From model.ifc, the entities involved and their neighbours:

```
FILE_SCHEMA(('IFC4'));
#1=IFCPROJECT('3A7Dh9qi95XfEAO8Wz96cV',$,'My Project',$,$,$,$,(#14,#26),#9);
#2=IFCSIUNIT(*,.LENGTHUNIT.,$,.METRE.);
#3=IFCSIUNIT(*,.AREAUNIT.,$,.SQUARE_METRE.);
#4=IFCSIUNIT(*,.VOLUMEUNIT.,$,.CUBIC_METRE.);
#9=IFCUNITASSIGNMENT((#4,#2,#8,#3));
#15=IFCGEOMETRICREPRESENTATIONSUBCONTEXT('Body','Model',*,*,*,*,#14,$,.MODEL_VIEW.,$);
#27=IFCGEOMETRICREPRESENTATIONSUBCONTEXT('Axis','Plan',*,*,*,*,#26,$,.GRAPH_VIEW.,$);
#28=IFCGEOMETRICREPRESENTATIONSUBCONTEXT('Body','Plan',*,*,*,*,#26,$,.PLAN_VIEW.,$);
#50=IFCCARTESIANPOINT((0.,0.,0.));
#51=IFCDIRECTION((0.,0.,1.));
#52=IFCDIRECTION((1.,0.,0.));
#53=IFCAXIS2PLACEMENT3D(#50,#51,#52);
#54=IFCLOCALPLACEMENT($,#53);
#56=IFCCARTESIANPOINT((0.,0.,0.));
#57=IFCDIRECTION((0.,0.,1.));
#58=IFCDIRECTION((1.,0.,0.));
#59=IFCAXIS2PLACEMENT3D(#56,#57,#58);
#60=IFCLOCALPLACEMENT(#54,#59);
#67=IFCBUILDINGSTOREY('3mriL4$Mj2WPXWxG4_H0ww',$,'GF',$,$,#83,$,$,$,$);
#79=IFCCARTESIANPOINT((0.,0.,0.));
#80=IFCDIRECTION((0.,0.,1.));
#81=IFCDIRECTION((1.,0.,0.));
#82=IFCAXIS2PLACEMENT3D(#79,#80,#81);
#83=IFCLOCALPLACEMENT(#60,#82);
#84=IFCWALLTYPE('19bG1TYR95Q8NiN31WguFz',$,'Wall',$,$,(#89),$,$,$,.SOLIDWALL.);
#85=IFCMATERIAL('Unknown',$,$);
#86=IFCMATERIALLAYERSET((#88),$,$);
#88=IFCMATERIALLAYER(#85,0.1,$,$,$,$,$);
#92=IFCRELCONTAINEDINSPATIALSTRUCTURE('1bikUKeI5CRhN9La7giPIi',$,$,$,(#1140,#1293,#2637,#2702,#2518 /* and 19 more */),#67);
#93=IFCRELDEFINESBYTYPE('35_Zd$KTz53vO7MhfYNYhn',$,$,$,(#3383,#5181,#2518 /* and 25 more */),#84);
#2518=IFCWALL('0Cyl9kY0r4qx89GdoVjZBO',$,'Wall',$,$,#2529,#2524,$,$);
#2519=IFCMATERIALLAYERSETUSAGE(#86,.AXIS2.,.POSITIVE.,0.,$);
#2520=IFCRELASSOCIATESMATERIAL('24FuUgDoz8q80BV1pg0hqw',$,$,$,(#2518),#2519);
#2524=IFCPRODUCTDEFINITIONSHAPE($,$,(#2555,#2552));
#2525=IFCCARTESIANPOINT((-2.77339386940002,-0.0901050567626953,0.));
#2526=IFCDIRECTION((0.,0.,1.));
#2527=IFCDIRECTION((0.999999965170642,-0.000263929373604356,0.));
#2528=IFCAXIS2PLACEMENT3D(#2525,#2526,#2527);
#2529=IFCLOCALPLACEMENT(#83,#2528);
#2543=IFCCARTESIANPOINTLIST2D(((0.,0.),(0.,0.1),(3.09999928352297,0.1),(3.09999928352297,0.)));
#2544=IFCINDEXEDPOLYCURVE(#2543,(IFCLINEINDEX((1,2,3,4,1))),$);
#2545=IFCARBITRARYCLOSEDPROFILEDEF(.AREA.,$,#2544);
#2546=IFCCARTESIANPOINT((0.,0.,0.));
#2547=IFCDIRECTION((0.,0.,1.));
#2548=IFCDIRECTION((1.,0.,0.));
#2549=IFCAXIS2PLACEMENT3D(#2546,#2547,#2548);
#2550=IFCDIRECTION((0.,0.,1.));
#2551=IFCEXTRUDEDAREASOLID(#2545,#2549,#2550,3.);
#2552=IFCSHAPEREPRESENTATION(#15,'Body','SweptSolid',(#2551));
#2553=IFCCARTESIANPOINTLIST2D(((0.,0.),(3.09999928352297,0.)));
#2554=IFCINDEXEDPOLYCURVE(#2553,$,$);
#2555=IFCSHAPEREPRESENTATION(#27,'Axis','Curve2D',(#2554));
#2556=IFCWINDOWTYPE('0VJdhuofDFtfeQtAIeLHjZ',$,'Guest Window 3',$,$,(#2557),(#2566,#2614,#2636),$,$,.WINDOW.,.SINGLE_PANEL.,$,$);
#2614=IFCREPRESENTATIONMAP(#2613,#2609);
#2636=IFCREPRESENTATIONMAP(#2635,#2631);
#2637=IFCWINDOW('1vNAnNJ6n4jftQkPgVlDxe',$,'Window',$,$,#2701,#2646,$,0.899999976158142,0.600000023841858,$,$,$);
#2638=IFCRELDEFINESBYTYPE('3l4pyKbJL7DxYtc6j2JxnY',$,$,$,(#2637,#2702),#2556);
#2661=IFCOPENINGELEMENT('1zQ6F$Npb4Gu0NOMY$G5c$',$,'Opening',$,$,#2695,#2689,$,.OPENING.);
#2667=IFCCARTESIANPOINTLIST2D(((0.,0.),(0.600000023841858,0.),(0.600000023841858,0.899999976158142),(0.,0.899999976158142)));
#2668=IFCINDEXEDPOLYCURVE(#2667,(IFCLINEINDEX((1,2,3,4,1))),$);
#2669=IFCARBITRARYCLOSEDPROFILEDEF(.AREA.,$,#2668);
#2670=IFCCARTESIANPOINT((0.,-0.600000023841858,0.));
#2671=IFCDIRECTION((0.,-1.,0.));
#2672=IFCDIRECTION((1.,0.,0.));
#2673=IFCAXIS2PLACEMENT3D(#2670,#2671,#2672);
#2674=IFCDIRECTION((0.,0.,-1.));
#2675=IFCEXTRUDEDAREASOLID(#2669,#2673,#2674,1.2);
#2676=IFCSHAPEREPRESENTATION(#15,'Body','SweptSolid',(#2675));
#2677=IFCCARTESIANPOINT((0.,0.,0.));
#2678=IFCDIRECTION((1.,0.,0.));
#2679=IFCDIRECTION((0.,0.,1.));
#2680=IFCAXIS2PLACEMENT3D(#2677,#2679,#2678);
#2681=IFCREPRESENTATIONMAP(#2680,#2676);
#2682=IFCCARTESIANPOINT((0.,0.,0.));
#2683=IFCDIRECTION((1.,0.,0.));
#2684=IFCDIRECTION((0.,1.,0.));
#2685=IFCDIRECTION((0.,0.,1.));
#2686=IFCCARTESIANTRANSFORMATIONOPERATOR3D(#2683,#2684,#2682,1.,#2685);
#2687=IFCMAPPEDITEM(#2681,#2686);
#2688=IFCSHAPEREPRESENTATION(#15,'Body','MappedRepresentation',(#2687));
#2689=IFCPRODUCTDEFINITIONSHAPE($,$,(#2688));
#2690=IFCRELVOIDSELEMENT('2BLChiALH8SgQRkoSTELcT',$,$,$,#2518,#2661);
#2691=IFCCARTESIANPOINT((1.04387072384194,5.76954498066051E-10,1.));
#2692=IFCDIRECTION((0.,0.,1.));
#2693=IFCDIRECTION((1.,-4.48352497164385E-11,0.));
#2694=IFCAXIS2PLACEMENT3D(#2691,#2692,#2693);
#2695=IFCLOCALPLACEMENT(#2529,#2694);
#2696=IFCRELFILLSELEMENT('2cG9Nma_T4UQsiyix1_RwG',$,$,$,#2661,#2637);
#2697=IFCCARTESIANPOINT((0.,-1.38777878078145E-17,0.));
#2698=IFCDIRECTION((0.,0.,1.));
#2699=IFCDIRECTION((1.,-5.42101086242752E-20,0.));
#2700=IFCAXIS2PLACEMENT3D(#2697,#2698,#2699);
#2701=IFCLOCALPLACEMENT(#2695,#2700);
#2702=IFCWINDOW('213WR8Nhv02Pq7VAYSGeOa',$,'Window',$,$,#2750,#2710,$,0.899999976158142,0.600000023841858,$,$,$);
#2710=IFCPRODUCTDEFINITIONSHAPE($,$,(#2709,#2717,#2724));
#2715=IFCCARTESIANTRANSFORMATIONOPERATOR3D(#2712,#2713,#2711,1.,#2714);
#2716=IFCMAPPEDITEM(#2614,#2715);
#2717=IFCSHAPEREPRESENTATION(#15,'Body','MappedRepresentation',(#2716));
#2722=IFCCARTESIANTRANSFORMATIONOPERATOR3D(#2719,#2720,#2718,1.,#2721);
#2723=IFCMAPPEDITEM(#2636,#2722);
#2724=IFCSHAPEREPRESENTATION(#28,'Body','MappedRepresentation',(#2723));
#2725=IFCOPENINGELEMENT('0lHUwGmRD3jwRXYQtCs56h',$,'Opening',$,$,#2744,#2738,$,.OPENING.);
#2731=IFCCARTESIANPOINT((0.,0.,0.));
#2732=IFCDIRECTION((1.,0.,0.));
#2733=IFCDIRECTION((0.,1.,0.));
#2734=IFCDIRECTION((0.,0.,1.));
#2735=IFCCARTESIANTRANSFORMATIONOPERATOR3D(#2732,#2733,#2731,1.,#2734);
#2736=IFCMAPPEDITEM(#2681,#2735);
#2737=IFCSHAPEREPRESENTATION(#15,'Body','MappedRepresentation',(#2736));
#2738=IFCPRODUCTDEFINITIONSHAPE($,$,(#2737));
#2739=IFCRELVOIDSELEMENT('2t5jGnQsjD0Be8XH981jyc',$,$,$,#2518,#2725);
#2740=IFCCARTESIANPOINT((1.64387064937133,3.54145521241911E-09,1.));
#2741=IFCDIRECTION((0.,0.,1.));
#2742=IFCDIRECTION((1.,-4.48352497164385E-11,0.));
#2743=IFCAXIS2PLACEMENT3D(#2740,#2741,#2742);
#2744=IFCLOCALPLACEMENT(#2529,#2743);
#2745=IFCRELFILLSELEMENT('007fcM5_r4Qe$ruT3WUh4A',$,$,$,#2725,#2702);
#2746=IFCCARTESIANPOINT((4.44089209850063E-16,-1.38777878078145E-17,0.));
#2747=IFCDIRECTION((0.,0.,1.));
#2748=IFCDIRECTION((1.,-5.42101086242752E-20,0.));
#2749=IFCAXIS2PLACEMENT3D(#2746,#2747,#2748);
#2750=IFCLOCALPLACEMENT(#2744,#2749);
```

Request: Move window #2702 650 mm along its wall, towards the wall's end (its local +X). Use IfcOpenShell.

```python
import ifcopenshell
import ifcopenshell.api.geometry
import ifcopenshell.util.placement

model = ifcopenshell.open("model.ifc")

window = model.by_guid("213WR8Nhv02Pq7VAYSGeOa")
opening = window.FillsVoids[0].RelatingOpeningElement
wall = opening.VoidsElements[0].RelatingBuildingElement

wall_matrix = ifcopenshell.util.placement.get_local_placement(wall.ObjectPlacement)
shift = wall_matrix[:3, 0] * 0.65
before = ifcopenshell.util.placement.get_local_placement(window.ObjectPlacement)[:3, 3].copy()

# The window is placed relative to its opening, so it follows when the opening moves.
matrix = ifcopenshell.util.placement.get_local_placement(opening.ObjectPlacement)
matrix[:3, 3] += shift
ifcopenshell.api.geometry.edit_object_placement(
    model, product=opening, matrix=matrix, is_si=False, should_transform_children=True
)

after = ifcopenshell.util.placement.get_local_placement(window.ObjectPlacement)[:3, 3]
print("window moved by", (after - before).round(3) + 0.0)

model.write("model_edited.ifc")
```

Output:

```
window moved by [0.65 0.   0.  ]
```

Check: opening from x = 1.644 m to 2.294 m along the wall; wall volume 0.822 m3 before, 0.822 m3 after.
